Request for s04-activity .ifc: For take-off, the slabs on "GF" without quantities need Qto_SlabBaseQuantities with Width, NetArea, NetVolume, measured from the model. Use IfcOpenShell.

First a look at what the model holds.

```python
import ifcopenshell
import ifcopenshell.util.element
import ifcopenshell.util.unit

model = ifcopenshell.open("s04-activity .ifc")
print(model.schema)
for unit_type in ("LENGTHUNIT", "AREAUNIT", "VOLUMEUNIT"):
    print(unit_type, ifcopenshell.util.unit.calculate_unit_scale(model, unit_type))
storey = next(s for s in model.by_type("IfcBuildingStorey") if s.Name == "GF")
slabs = [e for e in ifcopenshell.util.element.get_decomposition(storey) if e.is_a("IfcSlab")]
for e in sorted(slabs, key=lambda e: e.id()):
    print(e.id(), e.is_a(), e.Name, list(ifcopenshell.util.element.get_psets(e, qtos_only=True)), sep=" | ")
```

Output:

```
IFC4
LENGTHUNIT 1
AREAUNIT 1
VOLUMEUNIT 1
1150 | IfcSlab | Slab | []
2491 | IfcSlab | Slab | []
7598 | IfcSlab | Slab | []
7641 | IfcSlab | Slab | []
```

```python
import ifcopenshell
import ifcopenshell.api.pset
import ifcopenshell.geom
import ifcopenshell.util.element
import ifcopenshell.util.shape
import ifcopenshell.util.unit

model = ifcopenshell.open("s04-activity .ifc")
unit_scale = ifcopenshell.util.unit.calculate_unit_scale(model)
area_scale = ifcopenshell.util.unit.calculate_unit_scale(model, "AREAUNIT")
volume_scale = ifcopenshell.util.unit.calculate_unit_scale(model, "VOLUMEUNIT")
settings = ifcopenshell.geom.settings()

storey = next(s for s in model.by_type("IfcBuildingStorey") if s.Name == "GF")
slabs = [e for e in ifcopenshell.util.element.get_decomposition(storey) if e.is_a("IfcSlab")]

for e in sorted(slabs, key=lambda e: e.id()):
    if ifcopenshell.util.element.get_psets(e, qtos_only=True, should_inherit=False):
        continue
    # Geometry comes back in metres, in the element's own axes.
    shape = ifcopenshell.geom.create_shape(settings, e)
    values = {
        "Width": ifcopenshell.util.shape.get_z(shape.geometry) / unit_scale,
        "NetArea": ifcopenshell.util.shape.get_footprint_area(shape.geometry) / area_scale,
        "NetVolume": ifcopenshell.util.shape.get_volume(shape.geometry) / volume_scale,
    }
    qto = ifcopenshell.api.pset.add_qto(model, product=e, name="Qto_SlabBaseQuantities")
    ifcopenshell.api.pset.edit_qto(model, qto=qto, properties=values)
    print(e.id(), {k: round(v, 3) for k, v in values.items()})

model.write("s04-activity _v2.ifc")
```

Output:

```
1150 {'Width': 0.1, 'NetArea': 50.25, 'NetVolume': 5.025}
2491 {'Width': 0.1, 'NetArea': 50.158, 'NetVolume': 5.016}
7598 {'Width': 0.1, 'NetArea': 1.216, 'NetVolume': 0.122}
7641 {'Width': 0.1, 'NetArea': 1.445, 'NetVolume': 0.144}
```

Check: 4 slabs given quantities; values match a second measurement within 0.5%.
